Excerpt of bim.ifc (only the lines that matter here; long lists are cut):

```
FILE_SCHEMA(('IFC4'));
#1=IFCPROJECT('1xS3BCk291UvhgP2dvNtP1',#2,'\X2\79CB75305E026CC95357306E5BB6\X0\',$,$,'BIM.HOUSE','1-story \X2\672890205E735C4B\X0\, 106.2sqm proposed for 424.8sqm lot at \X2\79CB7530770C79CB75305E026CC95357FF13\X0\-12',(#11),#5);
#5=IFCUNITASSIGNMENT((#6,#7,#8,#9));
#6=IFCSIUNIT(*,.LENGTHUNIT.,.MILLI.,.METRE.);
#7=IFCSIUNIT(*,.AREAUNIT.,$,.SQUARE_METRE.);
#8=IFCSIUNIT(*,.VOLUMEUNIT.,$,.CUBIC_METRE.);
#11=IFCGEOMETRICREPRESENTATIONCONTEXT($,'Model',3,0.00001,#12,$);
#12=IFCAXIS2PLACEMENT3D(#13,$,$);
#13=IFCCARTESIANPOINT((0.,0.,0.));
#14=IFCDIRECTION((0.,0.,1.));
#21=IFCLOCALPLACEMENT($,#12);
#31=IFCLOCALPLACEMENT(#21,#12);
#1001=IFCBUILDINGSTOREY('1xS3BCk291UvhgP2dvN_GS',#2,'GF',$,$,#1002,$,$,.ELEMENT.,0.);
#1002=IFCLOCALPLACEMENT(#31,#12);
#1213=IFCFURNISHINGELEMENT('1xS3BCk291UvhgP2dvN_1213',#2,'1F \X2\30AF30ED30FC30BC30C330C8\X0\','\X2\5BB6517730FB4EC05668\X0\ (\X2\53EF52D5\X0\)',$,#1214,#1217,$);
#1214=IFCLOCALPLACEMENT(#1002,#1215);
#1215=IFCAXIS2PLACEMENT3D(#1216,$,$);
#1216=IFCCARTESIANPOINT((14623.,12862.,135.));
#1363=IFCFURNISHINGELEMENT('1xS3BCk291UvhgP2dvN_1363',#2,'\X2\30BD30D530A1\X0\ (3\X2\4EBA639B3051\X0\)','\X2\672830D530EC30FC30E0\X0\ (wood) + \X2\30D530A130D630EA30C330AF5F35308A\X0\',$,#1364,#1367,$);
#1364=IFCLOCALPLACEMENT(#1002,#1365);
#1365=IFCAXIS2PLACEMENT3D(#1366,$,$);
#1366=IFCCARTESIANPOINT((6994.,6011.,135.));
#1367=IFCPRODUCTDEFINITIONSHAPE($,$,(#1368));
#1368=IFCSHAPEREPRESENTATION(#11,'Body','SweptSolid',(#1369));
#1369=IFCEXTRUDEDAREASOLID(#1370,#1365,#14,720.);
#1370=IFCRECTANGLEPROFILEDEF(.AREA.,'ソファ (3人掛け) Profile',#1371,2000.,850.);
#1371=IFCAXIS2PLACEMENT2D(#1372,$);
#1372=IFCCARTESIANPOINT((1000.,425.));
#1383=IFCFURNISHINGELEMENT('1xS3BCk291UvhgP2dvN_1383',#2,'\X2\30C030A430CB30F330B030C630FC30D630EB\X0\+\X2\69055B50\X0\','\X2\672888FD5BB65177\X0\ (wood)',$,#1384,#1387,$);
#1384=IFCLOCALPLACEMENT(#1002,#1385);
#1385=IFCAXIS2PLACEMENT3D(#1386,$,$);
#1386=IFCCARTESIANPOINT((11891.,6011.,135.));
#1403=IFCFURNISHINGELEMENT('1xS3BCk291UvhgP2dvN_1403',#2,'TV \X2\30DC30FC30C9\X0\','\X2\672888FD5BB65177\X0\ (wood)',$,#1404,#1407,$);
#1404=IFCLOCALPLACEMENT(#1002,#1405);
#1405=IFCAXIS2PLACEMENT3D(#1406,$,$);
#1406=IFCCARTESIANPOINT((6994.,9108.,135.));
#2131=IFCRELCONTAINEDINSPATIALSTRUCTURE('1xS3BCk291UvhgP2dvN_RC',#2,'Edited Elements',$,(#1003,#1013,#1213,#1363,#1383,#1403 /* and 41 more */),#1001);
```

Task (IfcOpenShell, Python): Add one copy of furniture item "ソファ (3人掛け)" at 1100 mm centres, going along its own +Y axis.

```python
import ifcopenshell
import ifcopenshell.api.geometry
import ifcopenshell.api.root
import ifcopenshell.util.element
import ifcopenshell.util.placement
import ifcopenshell.util.unit

model = ifcopenshell.open("bim.ifc")
unit_scale = ifcopenshell.util.unit.calculate_unit_scale(model)


def reuse_history(source, copy):
    """copy_class also copies each property set's owner history, people and application; keep the originals."""
    for rel in copy.IsDefinedBy:
        if rel.is_a("IfcRelDefinesByProperties") and (history := rel.RelatingPropertyDefinition.OwnerHistory):
            rel.RelatingPropertyDefinition.OwnerHistory = source.OwnerHistory
            ifcopenshell.util.element.remove_deep2(model, history)


source = model.by_guid("1xS3BCk291UvhgP2dvN_1363")
base = ifcopenshell.util.placement.get_local_placement(source.ObjectPlacement)
step = base[:3, 1] * 1.1 / unit_scale

for i in range(1, 2):
    copy = ifcopenshell.api.root.copy_class(model, product=source)
    copy.Representation = ifcopenshell.util.element.copy_deep(
        model, source.Representation, exclude=["IfcGeometricRepresentationContext", "IfcRepresentationMap"]
    )
    reuse_history(source, copy)
    matrix = base.copy()
    matrix[:3, 3] += i * step
    print("added at", matrix[:3, 3].round(3) + 0.0)
    ifcopenshell.api.geometry.edit_object_placement(model, product=copy, matrix=matrix, is_si=False)

model.write("bim_rev.ifc")
```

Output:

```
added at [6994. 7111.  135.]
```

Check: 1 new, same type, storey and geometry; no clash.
